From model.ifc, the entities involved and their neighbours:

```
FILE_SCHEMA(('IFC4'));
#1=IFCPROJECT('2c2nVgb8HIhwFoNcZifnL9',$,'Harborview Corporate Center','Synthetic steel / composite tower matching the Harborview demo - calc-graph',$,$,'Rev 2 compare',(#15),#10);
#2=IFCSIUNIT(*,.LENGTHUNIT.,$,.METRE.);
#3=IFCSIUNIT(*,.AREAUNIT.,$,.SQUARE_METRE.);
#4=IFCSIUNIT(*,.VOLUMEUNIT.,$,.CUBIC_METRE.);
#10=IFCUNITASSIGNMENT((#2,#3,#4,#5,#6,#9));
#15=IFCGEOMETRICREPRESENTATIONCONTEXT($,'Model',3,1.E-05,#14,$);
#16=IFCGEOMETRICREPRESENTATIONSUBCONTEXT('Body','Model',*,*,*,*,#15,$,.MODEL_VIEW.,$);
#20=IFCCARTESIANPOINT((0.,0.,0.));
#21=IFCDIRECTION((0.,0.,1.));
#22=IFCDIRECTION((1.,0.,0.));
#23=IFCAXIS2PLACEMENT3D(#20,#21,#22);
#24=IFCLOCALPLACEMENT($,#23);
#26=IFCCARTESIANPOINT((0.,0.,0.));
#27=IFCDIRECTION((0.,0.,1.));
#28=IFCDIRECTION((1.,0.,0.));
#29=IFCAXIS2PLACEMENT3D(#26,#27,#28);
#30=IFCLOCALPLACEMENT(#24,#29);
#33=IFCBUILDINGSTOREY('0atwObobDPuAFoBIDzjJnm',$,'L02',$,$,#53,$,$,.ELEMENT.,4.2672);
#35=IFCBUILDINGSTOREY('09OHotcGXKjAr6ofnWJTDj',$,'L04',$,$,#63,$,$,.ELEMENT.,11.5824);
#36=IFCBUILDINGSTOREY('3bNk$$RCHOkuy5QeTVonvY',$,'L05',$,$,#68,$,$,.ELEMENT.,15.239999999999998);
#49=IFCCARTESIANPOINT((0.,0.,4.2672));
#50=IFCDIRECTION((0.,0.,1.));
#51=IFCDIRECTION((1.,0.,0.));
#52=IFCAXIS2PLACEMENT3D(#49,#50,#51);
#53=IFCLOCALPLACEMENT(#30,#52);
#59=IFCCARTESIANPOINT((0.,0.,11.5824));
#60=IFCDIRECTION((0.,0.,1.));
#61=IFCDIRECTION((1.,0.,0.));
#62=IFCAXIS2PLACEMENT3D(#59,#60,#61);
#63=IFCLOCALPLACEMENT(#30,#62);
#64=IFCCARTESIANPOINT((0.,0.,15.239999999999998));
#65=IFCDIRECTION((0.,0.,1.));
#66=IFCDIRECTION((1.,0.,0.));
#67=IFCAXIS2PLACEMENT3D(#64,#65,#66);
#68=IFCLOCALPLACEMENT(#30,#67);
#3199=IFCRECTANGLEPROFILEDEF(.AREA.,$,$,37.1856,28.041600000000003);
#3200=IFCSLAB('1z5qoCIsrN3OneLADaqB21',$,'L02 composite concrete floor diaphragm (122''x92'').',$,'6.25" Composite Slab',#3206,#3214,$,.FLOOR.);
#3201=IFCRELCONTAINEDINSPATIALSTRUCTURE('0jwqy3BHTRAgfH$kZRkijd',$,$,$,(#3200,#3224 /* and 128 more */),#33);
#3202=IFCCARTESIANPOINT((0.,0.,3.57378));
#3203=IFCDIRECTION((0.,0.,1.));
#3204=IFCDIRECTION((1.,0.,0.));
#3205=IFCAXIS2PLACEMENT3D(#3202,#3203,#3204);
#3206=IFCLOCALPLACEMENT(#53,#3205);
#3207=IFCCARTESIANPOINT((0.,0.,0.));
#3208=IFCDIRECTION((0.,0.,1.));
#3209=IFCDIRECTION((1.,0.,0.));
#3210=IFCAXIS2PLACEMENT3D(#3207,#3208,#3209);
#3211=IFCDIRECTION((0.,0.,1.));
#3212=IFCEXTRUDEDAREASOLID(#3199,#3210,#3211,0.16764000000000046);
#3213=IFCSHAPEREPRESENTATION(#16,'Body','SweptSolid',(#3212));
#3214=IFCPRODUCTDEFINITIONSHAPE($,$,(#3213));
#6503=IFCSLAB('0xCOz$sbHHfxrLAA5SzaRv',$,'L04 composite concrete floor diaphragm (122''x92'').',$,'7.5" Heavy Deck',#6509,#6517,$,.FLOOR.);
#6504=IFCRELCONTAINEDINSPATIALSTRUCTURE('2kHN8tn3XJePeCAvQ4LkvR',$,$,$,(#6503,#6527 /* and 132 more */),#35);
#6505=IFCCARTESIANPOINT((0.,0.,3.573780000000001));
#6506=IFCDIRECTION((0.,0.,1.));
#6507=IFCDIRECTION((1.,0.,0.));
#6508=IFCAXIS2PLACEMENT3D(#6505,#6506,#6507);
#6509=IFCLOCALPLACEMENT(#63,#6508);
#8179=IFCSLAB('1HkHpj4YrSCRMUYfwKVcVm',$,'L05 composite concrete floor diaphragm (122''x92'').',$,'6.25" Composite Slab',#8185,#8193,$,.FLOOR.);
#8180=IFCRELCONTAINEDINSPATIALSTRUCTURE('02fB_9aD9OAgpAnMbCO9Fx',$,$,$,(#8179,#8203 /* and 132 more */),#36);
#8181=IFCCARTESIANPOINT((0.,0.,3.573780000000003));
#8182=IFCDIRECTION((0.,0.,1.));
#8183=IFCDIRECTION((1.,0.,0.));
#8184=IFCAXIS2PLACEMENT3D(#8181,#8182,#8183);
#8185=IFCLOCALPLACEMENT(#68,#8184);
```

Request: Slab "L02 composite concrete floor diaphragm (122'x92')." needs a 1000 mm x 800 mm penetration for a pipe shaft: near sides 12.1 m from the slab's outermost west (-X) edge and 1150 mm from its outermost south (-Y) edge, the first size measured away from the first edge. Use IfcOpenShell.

```python
import numpy as np
import ifcopenshell
import ifcopenshell.api.feature
import ifcopenshell.api.geometry
import ifcopenshell.api.root
import ifcopenshell.geom
import ifcopenshell.util.placement
import ifcopenshell.util.representation
import ifcopenshell.util.shape
import ifcopenshell.util.unit

model = ifcopenshell.open("model.ifc")
unit_scale = ifcopenshell.util.unit.calculate_unit_scale(model)
settings = ifcopenshell.geom.settings()


def volume(element):
    """Net volume in cubic metres, openings subtracted."""
    shape = ifcopenshell.geom.create_shape(settings, element)
    return ifcopenshell.util.shape.get_volume(shape.geometry)


slab = model.by_guid("1z5qoCIsrN3OneLADaqB21")
before = volume(slab)

# Extent in the slab's own axes, in metres. The edges named are its -X and -Y sides.
slab_shape = ifcopenshell.geom.create_shape(settings, slab)
vertices = ifcopenshell.util.shape.get_vertices(slab_shape.geometry)
x_min, y_min, bottom = vertices.min(axis=0)
top = vertices[:, 2].max()

opening = ifcopenshell.api.root.create_entity(model, ifc_class="IfcOpeningElement", name="Pipe shaft opening", predefined_type="OPENING")
context = ifcopenshell.util.representation.get_context(model, "Model", "Body", "MODEL_VIEW")
width, depth = 1, 0.8
outline = [(0.0, 0.0), (width, 0.0), (width, depth), (0.0, depth), (0.0, 0.0)]
# Overshoot both faces by 50 mm so the cut is clean.
shape = ifcopenshell.api.geometry.add_slab_representation(
    model, context=context, depth=top - bottom + 0.1, polyline=outline
)
ifcopenshell.api.geometry.assign_representation(model, product=opening, representation=shape)

matrix = ifcopenshell.util.placement.get_local_placement(slab.ObjectPlacement)
matrix[:, 3] = matrix @ np.append(np.array([x_min + 12.1, y_min + 1.15, bottom - 0.05]) / unit_scale, 1.0)
ifcopenshell.api.geometry.edit_object_placement(model, product=opening, matrix=matrix, is_si=False)
ifcopenshell.api.feature.add_feature(model, feature=opening, element=slab)

after = volume(slab)

print(f"slab volume {before:.3f} -> {after:.3f} m3")

model.write("model_updated.ifc")
```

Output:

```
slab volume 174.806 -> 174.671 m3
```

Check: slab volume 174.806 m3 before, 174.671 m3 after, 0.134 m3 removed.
